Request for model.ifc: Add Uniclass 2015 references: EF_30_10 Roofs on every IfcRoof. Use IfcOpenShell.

First a look at what the model holds.

```python
import ifcopenshell

model = ifcopenshell.open("model.ifc")
print(model.schema)
print("classifications:", [c.Name for c in model.by_type("IfcClassification")])
for ifc_class in ("IfcDoor", "IfcRoof", "IfcStair", "IfcWall", "IfcWindow"):
    print(ifc_class, len(model.by_type(ifc_class)))
```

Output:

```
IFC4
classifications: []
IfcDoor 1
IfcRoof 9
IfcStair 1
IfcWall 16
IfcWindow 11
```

```python
import ifcopenshell
import ifcopenshell.api.classification

model = ifcopenshell.open("model.ifc")

system = ifcopenshell.api.classification.add_classification(model, classification="Uniclass 2015")

codes = {
    "IfcRoof": ("EF_30_10", "Roofs"),
}
for ifc_class, (code, name) in codes.items():
    products = model.by_type(ifc_class)
    ifcopenshell.api.classification.add_reference(
        model, products=products, classification=system, identification=code, name=name
    )
    print(code, len(products))

model.write("model_updated.ifc")
```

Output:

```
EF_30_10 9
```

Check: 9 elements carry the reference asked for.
